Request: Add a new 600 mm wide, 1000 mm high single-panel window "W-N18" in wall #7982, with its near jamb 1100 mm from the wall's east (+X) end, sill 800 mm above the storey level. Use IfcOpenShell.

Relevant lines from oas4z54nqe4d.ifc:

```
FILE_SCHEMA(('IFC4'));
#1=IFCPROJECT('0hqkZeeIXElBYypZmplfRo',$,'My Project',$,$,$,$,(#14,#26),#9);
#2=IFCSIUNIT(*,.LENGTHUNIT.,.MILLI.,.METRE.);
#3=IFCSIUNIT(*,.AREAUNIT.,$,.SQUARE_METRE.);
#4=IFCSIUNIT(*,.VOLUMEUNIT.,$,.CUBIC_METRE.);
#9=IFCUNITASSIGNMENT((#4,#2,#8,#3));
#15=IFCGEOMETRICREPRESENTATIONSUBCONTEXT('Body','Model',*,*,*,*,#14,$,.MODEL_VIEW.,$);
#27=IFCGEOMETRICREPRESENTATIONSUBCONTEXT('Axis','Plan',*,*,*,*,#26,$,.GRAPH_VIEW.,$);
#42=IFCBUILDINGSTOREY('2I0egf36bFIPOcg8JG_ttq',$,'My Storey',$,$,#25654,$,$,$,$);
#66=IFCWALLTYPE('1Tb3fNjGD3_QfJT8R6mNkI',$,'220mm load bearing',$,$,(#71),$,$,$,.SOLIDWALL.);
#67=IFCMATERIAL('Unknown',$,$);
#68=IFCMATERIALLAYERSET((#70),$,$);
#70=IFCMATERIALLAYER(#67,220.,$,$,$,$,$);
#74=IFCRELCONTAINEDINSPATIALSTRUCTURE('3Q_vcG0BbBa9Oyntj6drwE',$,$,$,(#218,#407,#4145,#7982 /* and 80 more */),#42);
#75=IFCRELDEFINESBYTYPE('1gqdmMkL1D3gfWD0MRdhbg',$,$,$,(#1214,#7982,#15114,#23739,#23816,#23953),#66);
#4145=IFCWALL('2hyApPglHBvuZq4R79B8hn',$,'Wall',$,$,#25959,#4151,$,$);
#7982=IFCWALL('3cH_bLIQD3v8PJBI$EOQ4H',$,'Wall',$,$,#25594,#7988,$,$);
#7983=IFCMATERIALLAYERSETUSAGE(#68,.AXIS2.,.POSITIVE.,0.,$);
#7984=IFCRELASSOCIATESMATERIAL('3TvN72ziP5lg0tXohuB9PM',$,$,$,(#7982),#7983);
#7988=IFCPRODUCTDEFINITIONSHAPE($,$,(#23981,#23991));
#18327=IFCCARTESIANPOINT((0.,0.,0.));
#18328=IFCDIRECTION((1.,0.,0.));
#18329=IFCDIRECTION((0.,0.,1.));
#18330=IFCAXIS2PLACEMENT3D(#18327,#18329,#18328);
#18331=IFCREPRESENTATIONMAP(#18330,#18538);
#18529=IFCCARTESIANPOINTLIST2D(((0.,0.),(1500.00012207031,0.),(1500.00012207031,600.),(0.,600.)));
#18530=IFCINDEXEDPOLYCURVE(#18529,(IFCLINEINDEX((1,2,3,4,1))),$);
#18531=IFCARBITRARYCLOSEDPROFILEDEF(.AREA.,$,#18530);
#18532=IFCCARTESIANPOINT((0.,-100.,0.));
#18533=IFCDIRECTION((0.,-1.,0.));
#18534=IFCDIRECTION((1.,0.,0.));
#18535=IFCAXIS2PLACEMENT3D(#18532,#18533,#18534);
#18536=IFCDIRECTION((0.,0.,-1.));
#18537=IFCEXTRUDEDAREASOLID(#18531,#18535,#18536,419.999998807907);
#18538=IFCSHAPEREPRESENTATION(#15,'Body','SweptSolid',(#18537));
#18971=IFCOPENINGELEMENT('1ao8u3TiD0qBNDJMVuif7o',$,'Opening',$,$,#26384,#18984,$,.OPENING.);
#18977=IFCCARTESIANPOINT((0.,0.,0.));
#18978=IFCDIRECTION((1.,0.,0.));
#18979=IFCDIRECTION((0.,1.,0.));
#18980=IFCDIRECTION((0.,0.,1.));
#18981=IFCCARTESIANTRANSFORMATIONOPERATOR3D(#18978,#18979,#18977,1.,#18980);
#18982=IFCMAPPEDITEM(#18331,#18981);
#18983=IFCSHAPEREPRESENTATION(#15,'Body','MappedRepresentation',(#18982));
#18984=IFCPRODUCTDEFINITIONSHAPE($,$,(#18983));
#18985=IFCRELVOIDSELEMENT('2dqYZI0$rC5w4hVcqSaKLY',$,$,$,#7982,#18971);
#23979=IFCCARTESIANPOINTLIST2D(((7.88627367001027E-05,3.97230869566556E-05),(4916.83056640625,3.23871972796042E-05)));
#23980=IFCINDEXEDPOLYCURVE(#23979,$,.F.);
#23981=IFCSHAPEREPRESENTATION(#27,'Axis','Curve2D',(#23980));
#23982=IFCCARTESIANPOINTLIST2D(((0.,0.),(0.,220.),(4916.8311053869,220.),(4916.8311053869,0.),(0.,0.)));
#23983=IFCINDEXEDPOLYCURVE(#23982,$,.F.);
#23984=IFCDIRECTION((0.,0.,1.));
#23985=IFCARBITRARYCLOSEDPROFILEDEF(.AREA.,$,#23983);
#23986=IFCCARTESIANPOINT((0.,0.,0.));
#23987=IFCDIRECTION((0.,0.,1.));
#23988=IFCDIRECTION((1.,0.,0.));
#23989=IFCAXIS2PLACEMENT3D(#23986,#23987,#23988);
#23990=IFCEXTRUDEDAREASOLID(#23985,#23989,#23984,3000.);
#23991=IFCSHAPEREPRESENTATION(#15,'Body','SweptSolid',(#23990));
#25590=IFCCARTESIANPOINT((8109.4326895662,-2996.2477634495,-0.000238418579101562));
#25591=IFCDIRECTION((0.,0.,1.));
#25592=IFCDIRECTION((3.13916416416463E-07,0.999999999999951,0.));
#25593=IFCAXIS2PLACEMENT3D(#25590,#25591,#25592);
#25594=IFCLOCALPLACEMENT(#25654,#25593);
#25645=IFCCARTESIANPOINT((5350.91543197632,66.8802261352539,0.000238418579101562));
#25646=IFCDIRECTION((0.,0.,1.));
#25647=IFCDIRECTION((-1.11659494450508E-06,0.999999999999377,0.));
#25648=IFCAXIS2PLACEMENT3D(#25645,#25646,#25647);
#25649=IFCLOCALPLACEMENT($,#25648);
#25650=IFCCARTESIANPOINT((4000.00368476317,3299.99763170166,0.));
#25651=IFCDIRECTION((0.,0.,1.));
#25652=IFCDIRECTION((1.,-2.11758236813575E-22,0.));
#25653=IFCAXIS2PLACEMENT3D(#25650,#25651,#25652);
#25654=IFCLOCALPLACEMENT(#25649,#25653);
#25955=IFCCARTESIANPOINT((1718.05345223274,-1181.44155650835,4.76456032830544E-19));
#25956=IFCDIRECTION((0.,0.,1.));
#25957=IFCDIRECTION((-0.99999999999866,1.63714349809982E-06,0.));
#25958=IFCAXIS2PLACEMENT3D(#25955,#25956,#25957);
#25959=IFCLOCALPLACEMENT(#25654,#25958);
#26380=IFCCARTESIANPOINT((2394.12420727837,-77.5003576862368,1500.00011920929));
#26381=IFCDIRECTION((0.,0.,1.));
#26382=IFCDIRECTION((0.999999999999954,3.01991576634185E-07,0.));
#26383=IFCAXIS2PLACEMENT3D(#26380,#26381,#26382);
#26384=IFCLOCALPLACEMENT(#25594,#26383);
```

```python
import numpy as np
import ifcopenshell
import ifcopenshell.api.feature
import ifcopenshell.api.geometry
import ifcopenshell.api.root
import ifcopenshell.api.spatial
import ifcopenshell.geom
import ifcopenshell.util.element
import ifcopenshell.util.placement
import ifcopenshell.util.representation
import ifcopenshell.util.shape
import ifcopenshell.util.unit

model = ifcopenshell.open("oas4z54nqe4d.ifc")
unit_scale = ifcopenshell.util.unit.calculate_unit_scale(model)
settings = ifcopenshell.geom.settings()


def volume(element):
    """Net volume in cubic metres, openings subtracted."""
    shape = ifcopenshell.geom.create_shape(settings, element)
    return ifcopenshell.util.shape.get_volume(shape.geometry)


wall = model.by_guid("3cH_bLIQD3v8PJBI$EOQ4H")
storey = ifcopenshell.util.element.get_container(wall, ifc_class="IfcBuildingStorey")
context = ifcopenshell.util.representation.get_context(model, "Model", "Body", "MODEL_VIEW")
before = volume(wall)

width, height, from_end, sill = 0.6, 1, 1.1, 0.8  # metres

# The wall runs along its own X axis, and the end named is its -X end.
wall_shape = ifcopenshell.geom.create_shape(settings, wall)
x, y, z = ifcopenshell.util.shape.get_vertices(wall_shape.geometry).T
start = x.min() + from_end
face, thickness = float(y.min()), float(y.max() - y.min())
wall_matrix = ifcopenshell.util.placement.get_local_placement(wall.ObjectPlacement)
level = ifcopenshell.util.placement.get_local_placement(storey.ObjectPlacement)[2, 3]


def in_wall(x, y):
    """Placement at x, y metres in the wall's axes, at sill height."""
    matrix = wall_matrix.copy()
    matrix[:, 3] = wall_matrix @ np.array([x / unit_scale, y / unit_scale, 0.0, 1.0])
    matrix[2, 3] = level + sill / unit_scale
    return matrix


# Opening: a box that overshoots both wall faces by 50 mm.
opening = ifcopenshell.api.root.create_entity(model, ifc_class="IfcOpeningElement", predefined_type="OPENING")
box = ifcopenshell.api.geometry.add_wall_representation(
    model, context=context, length=width, height=height, thickness=thickness + 0.1
)
ifcopenshell.api.geometry.assign_representation(model, product=opening, representation=box)
ifcopenshell.api.geometry.edit_object_placement(model, product=opening, matrix=in_wall(start, face - 0.05), is_si=False)
ifcopenshell.api.feature.add_feature(model, feature=opening, element=wall)

window = ifcopenshell.api.root.create_entity(model, ifc_class="IfcWindow", name="W-N18", predefined_type="WINDOW")
window.OverallWidth, window.OverallHeight = width / unit_scale, height / unit_scale
window.PartitioningType = "SINGLE_PANEL"
body = ifcopenshell.api.geometry.add_window_representation(
    model,
    context=context,
    overall_width=window.OverallWidth,
    overall_height=window.OverallHeight,
    partition_type="SINGLE_PANEL",
)
ifcopenshell.api.geometry.assign_representation(model, product=window, representation=body)
ifcopenshell.api.spatial.assign_container(model, products=[window], relating_structure=storey)
ifcopenshell.api.feature.add_filling(model, opening=opening, element=window)

# Centre the window in the wall's thickness.
ifcopenshell.api.geometry.edit_object_placement(model, product=window, matrix=in_wall(start, face), is_si=False)
window_shape = ifcopenshell.geom.create_shape(settings, window)
depth = ifcopenshell.util.shape.get_vertices(window_shape.geometry)[:, 1]
offset = face + thickness / 2 - (depth.min() + depth.max()) / 2
ifcopenshell.api.geometry.edit_object_placement(model, product=window, matrix=in_wall(start, offset), is_si=False)

after = volume(wall)

print(f"wall volume {before:.3f} -> {after:.3f} m3")

model.write("oas4z54nqe4d_rev.ifc")
```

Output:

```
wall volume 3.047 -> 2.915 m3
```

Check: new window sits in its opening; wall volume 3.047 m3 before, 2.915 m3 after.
